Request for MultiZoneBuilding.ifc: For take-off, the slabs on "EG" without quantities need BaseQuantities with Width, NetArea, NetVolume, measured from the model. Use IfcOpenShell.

First a look at what the model holds.

```python
import ifcopenshell
import ifcopenshell.util.element
import ifcopenshell.util.unit

model = ifcopenshell.open("MultiZoneBuilding.ifc")
print(model.schema)
for unit_type in ("LENGTHUNIT", "AREAUNIT", "VOLUMEUNIT"):
    print(unit_type, ifcopenshell.util.unit.calculate_unit_scale(model, unit_type))
storey = next(s for s in model.by_type("IfcBuildingStorey") if s.Name == "EG")
slabs = [e for e in ifcopenshell.util.element.get_decomposition(storey) if e.is_a("IfcSlab")]
for e in sorted(slabs, key=lambda e: e.id()):
    print(e.id(), e.is_a(), e.Name, list(ifcopenshell.util.element.get_psets(e, qtos_only=True)), sep=" | ")
```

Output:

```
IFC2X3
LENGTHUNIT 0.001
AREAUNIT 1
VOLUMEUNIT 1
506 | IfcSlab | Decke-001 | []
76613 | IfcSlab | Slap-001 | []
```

```python
import ifcopenshell
import ifcopenshell.api.pset
import ifcopenshell.geom
import ifcopenshell.util.element
import ifcopenshell.util.shape
import ifcopenshell.util.unit

model = ifcopenshell.open("MultiZoneBuilding.ifc")
unit_scale = ifcopenshell.util.unit.calculate_unit_scale(model)
area_scale = ifcopenshell.util.unit.calculate_unit_scale(model, "AREAUNIT")
volume_scale = ifcopenshell.util.unit.calculate_unit_scale(model, "VOLUMEUNIT")
settings = ifcopenshell.geom.settings()

storey = next(s for s in model.by_type("IfcBuildingStorey") if s.Name == "EG")
slabs = [e for e in ifcopenshell.util.element.get_decomposition(storey) if e.is_a("IfcSlab")]

for e in sorted(slabs, key=lambda e: e.id()):
    if ifcopenshell.util.element.get_psets(e, qtos_only=True, should_inherit=False):
        continue
    # Geometry comes back in metres, in the element's own axes.
    shape = ifcopenshell.geom.create_shape(settings, e)
    values = {
        "Width": ifcopenshell.util.shape.get_z(shape.geometry) / unit_scale,
        "NetArea": ifcopenshell.util.shape.get_footprint_area(shape.geometry) / area_scale,
        "NetVolume": ifcopenshell.util.shape.get_volume(shape.geometry) / volume_scale,
    }
    qto = ifcopenshell.api.pset.add_qto(model, product=e, name="BaseQuantities")
    ifcopenshell.api.pset.edit_qto(model, qto=qto, properties=values)
    print(e.id(), {k: round(v, 3) for k, v in values.items()})

model.write("MultiZoneBuilding_rev.ifc")
```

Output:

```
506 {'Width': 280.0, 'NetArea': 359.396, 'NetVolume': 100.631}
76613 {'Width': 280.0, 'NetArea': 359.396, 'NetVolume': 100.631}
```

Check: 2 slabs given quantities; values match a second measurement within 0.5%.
